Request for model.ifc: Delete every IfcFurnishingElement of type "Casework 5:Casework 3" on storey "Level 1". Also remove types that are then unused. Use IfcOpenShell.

First a look at what the model holds.

```python
import ifcopenshell
import ifcopenshell.util.element

model = ifcopenshell.open("model.ifc")
print(model.schema)
storey = next(s for s in model.by_type("IfcBuildingStorey") if s.Name == "Level 1")
furniture = [e for e in ifcopenshell.util.element.get_decomposition(storey) if e.is_a("IfcFurnishingElement")]
seen = {}
for e in furniture:
    element_type = ifcopenshell.util.element.get_type(e)
    name = element_type.Name if element_type not in (None, e) else None
    seen[name] = seen.get(name, 0) + 1
for name, count in sorted(seen.items(), key=str):
    print(count, "x", name)
```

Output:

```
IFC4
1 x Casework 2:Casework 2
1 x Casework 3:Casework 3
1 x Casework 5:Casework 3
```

```python
import ifcopenshell
import ifcopenshell.api.root
import ifcopenshell.util.element

model = ifcopenshell.open("model.ifc")

storey = next(s for s in model.by_type("IfcBuildingStorey") if s.Name == "Level 1")
furniture = [e for e in ifcopenshell.util.element.get_decomposition(storey) if e.is_a("IfcFurnishingElement")]
targets = [e for e in furniture if (t := ifcopenshell.util.element.get_type(e)) not in (None, e) and t.Name == "Casework 5:Casework 3"]
types = {ifcopenshell.util.element.get_type(e) for e in targets} - {None, *targets}

for e in targets:
    ifcopenshell.api.root.remove_product(model, product=e)
print(len(targets), "removed")

unused = [t for t in types if not ifcopenshell.util.element.get_types(t)]
for t in unused:
    ifcopenshell.api.root.remove_product(model, product=t)
print(len(unused), "unused types removed")

model.write("model_rev.ifc")
```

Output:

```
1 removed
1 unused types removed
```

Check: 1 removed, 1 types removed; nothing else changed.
